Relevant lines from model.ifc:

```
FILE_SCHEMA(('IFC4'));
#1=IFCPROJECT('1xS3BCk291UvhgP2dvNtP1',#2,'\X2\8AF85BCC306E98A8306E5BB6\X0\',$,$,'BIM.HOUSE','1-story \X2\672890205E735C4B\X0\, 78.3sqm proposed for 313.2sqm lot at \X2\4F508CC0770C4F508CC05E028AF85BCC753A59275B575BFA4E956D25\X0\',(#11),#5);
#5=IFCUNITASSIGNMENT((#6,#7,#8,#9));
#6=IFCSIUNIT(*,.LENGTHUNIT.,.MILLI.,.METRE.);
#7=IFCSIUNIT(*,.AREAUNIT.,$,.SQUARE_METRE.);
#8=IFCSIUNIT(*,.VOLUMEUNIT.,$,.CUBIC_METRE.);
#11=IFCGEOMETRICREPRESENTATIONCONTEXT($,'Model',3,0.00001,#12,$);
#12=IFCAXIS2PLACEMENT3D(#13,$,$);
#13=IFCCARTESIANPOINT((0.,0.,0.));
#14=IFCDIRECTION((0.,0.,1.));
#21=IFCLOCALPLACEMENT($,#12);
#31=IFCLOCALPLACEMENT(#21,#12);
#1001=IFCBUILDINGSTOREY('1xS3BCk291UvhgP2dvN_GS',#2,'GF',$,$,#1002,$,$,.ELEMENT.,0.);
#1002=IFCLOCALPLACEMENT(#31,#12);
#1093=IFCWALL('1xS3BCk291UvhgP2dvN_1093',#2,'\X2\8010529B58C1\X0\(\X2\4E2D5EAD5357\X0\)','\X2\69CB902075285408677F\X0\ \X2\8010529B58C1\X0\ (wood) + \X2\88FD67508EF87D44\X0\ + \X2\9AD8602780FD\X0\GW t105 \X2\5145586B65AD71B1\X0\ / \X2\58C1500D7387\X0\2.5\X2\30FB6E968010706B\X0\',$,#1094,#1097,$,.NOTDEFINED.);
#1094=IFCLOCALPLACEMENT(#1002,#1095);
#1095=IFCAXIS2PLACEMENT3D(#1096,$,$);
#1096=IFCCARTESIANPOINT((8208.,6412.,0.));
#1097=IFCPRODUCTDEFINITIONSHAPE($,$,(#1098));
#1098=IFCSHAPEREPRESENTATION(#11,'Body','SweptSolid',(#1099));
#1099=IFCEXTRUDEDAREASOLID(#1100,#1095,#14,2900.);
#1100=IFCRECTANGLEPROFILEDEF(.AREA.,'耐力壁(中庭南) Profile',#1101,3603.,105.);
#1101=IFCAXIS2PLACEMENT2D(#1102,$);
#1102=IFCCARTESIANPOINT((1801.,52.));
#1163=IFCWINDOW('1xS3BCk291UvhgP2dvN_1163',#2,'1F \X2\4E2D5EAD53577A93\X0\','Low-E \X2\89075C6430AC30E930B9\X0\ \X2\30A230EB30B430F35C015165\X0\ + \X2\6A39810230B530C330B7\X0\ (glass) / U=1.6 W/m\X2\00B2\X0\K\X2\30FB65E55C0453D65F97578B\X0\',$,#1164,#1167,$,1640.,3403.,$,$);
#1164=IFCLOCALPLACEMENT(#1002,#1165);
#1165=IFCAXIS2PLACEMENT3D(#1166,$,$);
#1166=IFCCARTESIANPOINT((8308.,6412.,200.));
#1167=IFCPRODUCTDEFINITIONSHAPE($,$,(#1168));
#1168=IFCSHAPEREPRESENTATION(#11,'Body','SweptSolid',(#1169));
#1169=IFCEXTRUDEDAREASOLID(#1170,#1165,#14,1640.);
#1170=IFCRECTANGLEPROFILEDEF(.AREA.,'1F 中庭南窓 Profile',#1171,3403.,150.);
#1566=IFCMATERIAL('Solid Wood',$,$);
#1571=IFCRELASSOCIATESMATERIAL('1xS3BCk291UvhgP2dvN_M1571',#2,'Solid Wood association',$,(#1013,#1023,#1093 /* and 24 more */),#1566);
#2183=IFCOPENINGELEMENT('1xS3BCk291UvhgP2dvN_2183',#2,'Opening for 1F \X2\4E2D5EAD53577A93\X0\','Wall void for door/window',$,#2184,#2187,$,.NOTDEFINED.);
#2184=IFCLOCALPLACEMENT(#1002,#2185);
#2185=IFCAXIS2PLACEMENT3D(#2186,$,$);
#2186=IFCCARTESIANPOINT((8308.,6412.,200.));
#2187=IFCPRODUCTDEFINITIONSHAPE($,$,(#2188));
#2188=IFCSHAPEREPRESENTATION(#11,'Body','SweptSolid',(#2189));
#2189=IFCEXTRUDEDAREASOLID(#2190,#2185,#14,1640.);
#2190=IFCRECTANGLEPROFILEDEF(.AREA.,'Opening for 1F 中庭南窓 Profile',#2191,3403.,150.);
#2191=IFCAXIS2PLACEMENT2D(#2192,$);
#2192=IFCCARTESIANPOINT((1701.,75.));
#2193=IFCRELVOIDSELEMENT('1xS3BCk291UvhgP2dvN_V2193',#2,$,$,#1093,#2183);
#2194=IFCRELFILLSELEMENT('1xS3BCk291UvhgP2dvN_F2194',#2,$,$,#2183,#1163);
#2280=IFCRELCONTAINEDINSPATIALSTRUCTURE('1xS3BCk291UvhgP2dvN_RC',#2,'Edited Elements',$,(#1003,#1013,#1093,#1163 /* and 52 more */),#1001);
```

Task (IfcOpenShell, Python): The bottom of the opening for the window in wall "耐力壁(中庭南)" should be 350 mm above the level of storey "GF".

```python
import numpy as np
import ifcopenshell
import ifcopenshell.api.geometry
import ifcopenshell.geom
import ifcopenshell.util.element
import ifcopenshell.util.placement
import ifcopenshell.util.shape
import ifcopenshell.util.unit

model = ifcopenshell.open("model.ifc")
unit_scale = ifcopenshell.util.unit.calculate_unit_scale(model)

window = model.by_id(1163)
opening = window.FillsVoids[0].RelatingOpeningElement
storey = ifcopenshell.util.element.get_container(window, ifc_class="IfcBuildingStorey")
level = ifcopenshell.util.placement.get_local_placement(storey.ObjectPlacement)[2, 3]

# The opening's origin need not be at the sill, so measure its lowest point.
shape = ifcopenshell.geom.create_shape(ifcopenshell.geom.settings(), opening)
bottom = ifcopenshell.util.shape.get_shape_bottom_elevation(shape, shape.geometry) / unit_scale
dz = level + 350.0 - bottom

shift = np.array([0.0, 0.0, dz])
# The window is not placed relative to its opening, so move both.
for product in (opening, window):
    matrix = ifcopenshell.util.placement.get_local_placement(product.ObjectPlacement)
    matrix[:3, 3] += shift
    ifcopenshell.api.geometry.edit_object_placement(model, product=product, matrix=matrix, is_si=False)

print(f"moved by {dz * unit_scale:+.3f} m")

model.write("model_edited.ifc")
```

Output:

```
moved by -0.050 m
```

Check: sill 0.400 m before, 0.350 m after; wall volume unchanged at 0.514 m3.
